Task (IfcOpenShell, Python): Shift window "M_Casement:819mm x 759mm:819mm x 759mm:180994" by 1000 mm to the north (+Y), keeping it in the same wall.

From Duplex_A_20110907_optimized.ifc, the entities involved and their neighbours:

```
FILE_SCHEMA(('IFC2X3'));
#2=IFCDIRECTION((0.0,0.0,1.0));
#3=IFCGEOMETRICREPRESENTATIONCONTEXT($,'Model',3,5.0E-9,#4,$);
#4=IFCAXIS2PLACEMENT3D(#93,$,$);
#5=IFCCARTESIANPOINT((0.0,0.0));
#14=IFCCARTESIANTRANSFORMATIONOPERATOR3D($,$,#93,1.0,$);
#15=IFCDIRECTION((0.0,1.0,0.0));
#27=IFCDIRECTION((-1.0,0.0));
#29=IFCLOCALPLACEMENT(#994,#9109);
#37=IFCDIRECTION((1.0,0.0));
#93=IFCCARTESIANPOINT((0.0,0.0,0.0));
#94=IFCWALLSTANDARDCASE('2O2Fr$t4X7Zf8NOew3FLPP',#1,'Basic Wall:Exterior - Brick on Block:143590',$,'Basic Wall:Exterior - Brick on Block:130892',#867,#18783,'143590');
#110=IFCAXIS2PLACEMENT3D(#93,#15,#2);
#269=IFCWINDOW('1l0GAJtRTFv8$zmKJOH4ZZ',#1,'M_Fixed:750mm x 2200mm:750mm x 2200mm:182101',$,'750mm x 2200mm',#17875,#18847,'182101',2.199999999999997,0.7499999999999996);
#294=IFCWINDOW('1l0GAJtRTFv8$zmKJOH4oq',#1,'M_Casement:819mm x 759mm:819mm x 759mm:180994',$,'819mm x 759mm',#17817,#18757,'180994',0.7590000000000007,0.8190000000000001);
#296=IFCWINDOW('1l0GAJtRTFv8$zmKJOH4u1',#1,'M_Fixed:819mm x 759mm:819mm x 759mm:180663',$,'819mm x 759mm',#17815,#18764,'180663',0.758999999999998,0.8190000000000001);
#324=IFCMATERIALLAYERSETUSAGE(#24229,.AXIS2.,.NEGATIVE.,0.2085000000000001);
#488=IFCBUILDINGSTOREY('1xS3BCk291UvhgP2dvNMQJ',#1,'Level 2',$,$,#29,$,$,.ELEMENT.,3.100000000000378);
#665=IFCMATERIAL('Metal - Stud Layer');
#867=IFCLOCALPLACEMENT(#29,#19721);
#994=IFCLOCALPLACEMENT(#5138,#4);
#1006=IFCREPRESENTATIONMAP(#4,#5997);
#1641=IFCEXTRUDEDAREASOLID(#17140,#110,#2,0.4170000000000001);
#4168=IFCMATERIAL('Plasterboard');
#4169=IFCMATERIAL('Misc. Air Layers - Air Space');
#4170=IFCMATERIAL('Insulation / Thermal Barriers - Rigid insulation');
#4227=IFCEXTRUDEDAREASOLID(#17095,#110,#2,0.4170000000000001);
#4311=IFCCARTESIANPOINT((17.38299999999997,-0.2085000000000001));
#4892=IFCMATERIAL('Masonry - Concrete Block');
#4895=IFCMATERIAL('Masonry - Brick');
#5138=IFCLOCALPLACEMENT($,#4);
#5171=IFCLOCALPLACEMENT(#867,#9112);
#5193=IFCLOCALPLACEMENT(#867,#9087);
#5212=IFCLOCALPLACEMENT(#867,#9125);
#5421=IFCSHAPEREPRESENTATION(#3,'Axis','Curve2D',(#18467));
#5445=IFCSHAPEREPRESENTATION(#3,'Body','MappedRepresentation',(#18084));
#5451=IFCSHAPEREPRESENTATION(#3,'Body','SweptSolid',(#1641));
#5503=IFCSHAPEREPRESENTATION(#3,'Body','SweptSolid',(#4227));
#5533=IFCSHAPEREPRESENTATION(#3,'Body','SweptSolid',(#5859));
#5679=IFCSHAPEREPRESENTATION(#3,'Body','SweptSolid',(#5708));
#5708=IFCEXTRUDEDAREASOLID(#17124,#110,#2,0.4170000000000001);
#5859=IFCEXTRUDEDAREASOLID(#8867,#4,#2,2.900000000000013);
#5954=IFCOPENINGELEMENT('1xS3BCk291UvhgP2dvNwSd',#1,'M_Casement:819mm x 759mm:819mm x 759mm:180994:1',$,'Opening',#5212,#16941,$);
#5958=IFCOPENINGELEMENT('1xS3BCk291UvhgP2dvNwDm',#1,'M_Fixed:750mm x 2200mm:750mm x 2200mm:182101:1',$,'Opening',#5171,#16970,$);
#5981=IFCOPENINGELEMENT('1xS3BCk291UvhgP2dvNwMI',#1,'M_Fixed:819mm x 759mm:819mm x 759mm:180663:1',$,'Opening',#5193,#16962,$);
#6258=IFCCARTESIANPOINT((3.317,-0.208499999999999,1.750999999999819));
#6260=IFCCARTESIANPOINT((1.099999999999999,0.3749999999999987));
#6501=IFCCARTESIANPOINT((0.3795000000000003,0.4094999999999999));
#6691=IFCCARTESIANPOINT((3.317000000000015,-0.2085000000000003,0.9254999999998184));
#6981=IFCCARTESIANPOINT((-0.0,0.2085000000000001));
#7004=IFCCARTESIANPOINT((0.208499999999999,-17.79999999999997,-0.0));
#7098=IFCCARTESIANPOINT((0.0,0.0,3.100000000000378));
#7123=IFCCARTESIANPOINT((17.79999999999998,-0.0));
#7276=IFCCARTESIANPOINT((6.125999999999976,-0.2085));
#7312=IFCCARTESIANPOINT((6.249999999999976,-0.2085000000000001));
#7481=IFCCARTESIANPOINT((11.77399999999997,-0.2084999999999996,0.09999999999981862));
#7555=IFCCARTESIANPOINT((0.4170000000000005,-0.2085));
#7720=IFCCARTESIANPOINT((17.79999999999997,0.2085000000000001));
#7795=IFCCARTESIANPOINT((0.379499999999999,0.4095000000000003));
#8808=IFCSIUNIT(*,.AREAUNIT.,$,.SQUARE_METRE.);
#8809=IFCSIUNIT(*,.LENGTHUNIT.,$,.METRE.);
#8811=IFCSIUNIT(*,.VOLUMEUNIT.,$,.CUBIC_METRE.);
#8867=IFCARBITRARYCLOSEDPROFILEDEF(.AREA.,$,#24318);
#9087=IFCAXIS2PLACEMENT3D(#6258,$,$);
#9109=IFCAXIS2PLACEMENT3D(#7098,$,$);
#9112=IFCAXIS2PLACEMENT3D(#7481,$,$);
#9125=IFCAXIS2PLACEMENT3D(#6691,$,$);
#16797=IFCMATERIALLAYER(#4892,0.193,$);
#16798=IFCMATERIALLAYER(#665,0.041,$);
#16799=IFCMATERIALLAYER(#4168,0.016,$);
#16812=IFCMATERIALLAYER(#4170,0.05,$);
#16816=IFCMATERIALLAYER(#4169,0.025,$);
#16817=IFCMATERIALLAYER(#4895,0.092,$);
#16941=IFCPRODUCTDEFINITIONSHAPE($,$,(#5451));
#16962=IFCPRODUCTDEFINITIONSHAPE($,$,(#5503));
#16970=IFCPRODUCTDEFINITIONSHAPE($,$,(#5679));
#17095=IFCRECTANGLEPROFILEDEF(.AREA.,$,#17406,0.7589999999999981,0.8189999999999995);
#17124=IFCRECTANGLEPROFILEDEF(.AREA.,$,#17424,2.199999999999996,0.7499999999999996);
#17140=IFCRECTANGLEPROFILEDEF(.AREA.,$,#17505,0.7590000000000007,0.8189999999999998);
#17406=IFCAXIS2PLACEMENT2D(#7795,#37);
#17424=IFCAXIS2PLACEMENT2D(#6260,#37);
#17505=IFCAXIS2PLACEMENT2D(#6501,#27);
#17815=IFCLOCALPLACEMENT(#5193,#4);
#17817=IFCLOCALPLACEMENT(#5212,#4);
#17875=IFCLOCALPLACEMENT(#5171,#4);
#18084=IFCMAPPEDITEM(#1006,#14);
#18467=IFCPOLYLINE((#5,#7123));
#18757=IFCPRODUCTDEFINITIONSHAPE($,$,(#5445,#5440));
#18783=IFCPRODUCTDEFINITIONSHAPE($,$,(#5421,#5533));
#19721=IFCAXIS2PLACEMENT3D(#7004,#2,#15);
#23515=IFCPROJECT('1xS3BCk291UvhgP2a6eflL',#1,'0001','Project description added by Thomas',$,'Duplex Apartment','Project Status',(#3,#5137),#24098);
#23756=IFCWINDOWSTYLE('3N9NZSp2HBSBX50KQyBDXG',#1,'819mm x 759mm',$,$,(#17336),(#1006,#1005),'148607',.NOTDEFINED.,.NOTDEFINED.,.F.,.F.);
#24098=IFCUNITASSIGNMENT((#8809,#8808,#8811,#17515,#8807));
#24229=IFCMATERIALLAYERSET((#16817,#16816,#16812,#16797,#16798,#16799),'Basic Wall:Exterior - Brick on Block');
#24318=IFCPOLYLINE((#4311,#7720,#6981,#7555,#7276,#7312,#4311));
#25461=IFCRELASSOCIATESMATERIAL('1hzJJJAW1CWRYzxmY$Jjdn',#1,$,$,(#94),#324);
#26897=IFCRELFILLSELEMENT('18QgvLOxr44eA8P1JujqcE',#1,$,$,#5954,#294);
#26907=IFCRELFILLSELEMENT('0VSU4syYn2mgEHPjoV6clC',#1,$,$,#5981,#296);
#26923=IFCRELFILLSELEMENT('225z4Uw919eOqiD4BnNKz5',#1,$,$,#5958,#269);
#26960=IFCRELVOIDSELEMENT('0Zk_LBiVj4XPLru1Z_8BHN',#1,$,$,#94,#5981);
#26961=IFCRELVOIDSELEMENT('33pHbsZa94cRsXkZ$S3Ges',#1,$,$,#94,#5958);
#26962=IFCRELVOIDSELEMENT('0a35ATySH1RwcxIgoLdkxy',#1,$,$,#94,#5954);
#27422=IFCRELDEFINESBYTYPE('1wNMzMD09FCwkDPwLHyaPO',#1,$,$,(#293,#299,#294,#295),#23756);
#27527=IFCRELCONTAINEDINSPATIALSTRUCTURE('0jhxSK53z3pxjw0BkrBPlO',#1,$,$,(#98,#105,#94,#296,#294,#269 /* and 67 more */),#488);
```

```python
import ifcopenshell
import ifcopenshell.api.geometry
import ifcopenshell.util.placement
import ifcopenshell.util.unit

model = ifcopenshell.open("Duplex_A_20110907_optimized.ifc")
unit_scale = ifcopenshell.util.unit.calculate_unit_scale(model)

window = model.by_guid("1l0GAJtRTFv8$zmKJOH4oq")
opening = window.FillsVoids[0].RelatingOpeningElement
wall = opening.VoidsElements[0].RelatingBuildingElement

wall_matrix = ifcopenshell.util.placement.get_local_placement(wall.ObjectPlacement)
shift = wall_matrix[:3, 0] * 1 / unit_scale
before = ifcopenshell.util.placement.get_local_placement(window.ObjectPlacement)[:3, 3].copy()

# The window is placed relative to its opening, so it follows when the opening moves.
matrix = ifcopenshell.util.placement.get_local_placement(opening.ObjectPlacement)
matrix[:3, 3] += shift
ifcopenshell.api.geometry.edit_object_placement(
    model, product=opening, matrix=matrix, is_si=False, should_transform_children=True
)

after = ifcopenshell.util.placement.get_local_placement(window.ObjectPlacement)[:3, 3]
print("window moved by", (after - before).round(3) + 0.0)

model.write("Duplex_A_20110907_optimized_updated.ifc")
```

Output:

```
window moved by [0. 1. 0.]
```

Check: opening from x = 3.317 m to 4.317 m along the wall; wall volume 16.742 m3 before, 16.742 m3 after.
